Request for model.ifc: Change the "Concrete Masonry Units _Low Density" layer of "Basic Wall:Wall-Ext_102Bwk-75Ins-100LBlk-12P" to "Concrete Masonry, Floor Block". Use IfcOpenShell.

First a look at what the model holds.

```python
import ifcopenshell
import ifcopenshell.util.element

model = ifcopenshell.open("model.ifc")
print(model.schema)
for layer_set in model.by_type("IfcMaterialLayerSet"):
    if layer_set.LayerSetName == "Basic Wall:Wall-Ext_102Bwk-75Ins-100LBlk-12P":
        for layer in layer_set.MaterialLayers:
            print(layer.id(), layer.Material and layer.Material.Name, layer.LayerThickness, sep=" | ")
        print(len(ifcopenshell.util.element.get_elements_by_material(model, layer_set)), "elements and types use it")
print(sorted(m.Name for m in model.by_type("IfcMaterial") if m.Name)[:60])
```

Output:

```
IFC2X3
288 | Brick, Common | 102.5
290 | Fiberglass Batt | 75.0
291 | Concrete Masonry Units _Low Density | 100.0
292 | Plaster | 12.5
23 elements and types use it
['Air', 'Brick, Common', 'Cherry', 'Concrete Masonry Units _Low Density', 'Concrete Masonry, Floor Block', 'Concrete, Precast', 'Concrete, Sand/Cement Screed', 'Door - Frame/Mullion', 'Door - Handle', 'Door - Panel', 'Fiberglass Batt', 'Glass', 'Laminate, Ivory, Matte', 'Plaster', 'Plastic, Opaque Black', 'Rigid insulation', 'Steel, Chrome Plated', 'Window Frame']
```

```python
import ifcopenshell
import ifcopenshell.api.material

model = ifcopenshell.open("model.ifc")

layer_set = next(s for s in model.by_type("IfcMaterialLayerSet") if s.LayerSetName == "Basic Wall:Wall-Ext_102Bwk-75Ins-100LBlk-12P")
layer = next(l for l in layer_set.MaterialLayers if l.Material and l.Material.Name == "Concrete Masonry Units _Low Density")
material = next(m for m in model.by_type("IfcMaterial") if m.Name == "Concrete Masonry, Floor Block")

# Point this one layer at the other material; renaming the old one would change it everywhere.
ifcopenshell.api.material.edit_layer(model, layer=layer, attributes={}, material=material)

print([l.Material.Name if l.Material else None for l in layer_set.MaterialLayers])

model.write("model_updated.ifc")
```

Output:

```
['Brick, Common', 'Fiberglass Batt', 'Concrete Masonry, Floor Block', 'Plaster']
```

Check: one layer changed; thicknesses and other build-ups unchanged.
